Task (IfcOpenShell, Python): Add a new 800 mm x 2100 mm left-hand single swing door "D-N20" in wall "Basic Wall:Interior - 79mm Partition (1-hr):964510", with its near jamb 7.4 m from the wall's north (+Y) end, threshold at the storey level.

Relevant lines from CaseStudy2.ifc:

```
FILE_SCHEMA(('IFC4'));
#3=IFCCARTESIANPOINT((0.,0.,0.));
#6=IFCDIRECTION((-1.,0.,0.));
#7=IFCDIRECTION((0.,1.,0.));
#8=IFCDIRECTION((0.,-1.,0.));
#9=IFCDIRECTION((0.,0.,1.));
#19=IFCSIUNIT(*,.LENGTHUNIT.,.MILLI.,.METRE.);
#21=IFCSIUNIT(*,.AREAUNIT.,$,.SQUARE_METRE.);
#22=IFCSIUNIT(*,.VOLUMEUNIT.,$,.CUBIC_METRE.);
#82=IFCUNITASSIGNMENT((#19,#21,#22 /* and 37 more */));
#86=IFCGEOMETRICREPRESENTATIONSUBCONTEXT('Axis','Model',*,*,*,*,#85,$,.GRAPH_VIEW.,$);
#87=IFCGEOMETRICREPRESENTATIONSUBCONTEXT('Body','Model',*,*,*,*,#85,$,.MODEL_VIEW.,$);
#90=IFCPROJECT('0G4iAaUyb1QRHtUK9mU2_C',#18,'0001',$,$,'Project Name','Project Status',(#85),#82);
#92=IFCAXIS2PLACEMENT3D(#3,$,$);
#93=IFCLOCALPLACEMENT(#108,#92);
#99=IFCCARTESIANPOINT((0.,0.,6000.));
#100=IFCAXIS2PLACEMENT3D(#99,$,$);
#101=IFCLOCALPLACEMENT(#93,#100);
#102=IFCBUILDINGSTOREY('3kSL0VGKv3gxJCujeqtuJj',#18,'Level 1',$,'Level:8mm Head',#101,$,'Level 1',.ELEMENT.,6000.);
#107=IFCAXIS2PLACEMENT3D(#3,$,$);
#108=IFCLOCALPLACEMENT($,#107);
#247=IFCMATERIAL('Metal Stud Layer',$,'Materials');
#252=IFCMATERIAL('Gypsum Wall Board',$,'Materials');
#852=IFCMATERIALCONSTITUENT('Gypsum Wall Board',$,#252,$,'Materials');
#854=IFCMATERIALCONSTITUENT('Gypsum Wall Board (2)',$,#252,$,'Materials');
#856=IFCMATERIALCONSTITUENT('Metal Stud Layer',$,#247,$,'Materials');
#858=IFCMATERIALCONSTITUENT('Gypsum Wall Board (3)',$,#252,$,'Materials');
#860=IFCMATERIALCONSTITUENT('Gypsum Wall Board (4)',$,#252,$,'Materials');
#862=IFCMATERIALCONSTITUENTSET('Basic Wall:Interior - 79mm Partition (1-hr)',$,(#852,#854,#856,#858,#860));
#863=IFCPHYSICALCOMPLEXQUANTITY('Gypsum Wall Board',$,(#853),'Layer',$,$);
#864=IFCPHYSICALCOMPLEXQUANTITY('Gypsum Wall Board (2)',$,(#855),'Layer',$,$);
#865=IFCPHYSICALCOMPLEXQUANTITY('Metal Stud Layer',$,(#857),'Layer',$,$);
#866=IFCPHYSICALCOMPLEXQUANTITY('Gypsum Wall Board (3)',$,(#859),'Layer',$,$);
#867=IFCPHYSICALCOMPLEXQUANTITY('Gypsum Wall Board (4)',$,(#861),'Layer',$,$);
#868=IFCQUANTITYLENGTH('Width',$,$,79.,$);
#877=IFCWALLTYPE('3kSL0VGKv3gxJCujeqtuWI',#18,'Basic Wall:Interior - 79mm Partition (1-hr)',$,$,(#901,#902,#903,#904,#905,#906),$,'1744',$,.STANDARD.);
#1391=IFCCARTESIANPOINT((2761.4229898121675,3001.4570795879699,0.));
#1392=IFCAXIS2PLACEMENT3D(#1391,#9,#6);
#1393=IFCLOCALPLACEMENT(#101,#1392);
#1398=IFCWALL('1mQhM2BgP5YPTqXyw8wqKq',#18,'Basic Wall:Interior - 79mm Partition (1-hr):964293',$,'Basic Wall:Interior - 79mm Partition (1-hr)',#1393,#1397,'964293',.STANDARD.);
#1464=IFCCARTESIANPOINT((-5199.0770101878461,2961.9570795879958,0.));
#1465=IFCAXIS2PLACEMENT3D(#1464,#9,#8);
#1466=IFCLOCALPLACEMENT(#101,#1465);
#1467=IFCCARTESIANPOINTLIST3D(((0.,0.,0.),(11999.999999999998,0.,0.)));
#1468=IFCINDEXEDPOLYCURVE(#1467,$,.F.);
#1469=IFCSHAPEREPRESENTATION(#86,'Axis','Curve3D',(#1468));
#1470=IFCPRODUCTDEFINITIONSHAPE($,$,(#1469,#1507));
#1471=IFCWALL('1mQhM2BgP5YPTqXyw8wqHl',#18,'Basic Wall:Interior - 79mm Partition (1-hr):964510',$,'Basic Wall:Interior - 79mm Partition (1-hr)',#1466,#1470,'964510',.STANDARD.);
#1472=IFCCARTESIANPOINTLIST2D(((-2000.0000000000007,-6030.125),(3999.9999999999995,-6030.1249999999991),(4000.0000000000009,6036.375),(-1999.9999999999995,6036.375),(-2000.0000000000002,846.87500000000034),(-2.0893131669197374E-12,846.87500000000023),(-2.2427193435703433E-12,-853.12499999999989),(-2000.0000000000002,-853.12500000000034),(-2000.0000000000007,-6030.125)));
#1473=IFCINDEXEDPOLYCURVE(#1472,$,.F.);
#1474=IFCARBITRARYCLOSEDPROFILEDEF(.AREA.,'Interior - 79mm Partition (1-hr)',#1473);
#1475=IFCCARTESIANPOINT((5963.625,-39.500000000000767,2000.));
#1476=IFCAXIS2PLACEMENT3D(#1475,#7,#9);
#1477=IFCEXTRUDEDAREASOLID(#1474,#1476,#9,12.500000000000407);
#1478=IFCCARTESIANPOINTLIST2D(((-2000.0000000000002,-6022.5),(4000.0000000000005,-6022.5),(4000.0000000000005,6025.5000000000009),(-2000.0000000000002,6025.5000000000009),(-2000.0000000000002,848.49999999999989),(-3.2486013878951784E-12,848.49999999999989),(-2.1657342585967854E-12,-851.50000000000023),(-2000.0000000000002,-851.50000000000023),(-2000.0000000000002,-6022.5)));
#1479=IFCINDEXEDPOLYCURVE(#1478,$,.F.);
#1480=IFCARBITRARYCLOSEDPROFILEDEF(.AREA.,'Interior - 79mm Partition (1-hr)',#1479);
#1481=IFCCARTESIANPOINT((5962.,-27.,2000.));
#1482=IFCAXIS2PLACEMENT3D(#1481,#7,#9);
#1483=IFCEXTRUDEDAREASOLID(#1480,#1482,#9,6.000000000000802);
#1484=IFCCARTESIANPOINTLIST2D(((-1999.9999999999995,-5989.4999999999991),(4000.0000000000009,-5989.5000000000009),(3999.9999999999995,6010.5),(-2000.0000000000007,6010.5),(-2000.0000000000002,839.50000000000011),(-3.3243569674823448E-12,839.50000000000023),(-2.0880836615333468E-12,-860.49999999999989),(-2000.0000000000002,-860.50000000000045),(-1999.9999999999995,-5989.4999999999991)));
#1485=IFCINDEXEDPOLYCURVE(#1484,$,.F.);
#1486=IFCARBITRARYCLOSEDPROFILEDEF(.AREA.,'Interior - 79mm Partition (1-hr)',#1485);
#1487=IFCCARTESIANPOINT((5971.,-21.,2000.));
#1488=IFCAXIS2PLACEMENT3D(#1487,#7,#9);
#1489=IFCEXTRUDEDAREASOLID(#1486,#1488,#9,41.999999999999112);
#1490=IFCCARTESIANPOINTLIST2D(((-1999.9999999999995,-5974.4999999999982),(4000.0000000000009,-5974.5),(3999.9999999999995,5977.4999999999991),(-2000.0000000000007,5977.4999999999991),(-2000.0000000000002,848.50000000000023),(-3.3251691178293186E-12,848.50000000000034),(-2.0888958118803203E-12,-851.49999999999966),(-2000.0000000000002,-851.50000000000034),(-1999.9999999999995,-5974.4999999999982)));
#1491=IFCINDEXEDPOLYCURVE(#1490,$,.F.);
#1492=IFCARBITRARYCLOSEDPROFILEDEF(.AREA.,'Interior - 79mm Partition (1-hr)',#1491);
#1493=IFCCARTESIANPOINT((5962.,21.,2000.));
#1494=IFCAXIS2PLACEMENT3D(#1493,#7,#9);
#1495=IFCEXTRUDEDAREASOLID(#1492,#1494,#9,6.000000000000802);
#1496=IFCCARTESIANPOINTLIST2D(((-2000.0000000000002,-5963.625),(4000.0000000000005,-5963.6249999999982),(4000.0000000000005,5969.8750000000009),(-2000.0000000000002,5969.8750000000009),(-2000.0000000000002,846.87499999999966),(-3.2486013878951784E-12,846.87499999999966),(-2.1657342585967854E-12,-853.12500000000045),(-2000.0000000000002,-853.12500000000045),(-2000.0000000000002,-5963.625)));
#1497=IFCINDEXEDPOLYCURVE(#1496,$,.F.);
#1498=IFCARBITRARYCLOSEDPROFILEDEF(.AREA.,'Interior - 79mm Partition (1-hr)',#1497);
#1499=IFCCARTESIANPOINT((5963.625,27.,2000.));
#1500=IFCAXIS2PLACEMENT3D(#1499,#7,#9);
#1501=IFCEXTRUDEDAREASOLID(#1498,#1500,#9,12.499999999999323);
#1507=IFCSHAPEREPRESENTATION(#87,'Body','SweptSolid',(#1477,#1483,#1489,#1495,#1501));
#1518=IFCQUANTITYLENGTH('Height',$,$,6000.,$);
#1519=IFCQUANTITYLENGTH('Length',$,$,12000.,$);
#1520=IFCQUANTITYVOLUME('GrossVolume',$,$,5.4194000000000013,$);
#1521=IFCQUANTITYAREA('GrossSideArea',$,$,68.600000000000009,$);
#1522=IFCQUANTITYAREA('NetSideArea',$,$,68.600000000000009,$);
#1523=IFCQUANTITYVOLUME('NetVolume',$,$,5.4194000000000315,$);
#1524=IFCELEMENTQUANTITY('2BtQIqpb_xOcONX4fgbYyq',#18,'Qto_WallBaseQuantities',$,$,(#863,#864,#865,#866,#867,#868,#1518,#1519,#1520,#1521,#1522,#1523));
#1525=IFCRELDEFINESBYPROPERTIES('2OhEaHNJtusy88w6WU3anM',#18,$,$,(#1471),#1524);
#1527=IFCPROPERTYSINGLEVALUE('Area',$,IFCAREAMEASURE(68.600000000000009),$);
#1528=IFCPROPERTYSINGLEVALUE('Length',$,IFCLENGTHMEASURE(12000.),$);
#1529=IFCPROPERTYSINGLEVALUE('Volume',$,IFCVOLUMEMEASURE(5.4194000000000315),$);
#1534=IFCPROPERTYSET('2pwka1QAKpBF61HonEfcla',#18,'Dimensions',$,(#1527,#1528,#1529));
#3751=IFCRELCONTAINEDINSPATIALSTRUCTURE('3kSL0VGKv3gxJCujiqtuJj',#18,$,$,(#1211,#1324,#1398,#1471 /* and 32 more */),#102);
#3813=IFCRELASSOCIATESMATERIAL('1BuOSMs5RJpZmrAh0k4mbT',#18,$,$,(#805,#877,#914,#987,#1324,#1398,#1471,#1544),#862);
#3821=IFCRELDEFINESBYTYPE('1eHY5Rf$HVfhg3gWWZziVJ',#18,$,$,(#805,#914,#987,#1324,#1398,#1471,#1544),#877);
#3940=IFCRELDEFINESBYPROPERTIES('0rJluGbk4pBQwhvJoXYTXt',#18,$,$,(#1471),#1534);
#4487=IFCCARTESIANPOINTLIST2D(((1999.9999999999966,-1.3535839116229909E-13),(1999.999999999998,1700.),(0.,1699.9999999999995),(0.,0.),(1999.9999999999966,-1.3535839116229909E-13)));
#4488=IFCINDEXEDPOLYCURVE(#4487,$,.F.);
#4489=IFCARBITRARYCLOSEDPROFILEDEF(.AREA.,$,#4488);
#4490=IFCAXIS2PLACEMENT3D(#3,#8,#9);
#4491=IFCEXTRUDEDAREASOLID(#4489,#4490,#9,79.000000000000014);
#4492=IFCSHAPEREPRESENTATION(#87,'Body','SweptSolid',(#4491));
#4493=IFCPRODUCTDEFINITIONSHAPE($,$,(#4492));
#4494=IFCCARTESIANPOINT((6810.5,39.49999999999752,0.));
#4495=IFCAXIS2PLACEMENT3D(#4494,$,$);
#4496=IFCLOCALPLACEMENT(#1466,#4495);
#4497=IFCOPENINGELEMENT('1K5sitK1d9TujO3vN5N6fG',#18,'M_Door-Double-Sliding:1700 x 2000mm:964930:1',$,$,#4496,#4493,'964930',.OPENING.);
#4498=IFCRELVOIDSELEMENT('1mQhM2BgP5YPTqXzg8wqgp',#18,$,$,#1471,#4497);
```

```python
import numpy as np
import ifcopenshell
import ifcopenshell.api.feature
import ifcopenshell.api.geometry
import ifcopenshell.api.pset
import ifcopenshell.api.root
import ifcopenshell.api.spatial
import ifcopenshell.geom
import ifcopenshell.util.element
import ifcopenshell.util.placement
import ifcopenshell.util.representation
import ifcopenshell.util.shape
import ifcopenshell.util.unit

model = ifcopenshell.open("CaseStudy2.ifc")
unit_scale = ifcopenshell.util.unit.calculate_unit_scale(model)
area_scale = ifcopenshell.util.unit.calculate_unit_scale(model, "AREAUNIT")
volume_scale = ifcopenshell.util.unit.calculate_unit_scale(model, "VOLUMEUNIT")
settings = ifcopenshell.geom.settings()


def volume(element):
    """Net volume in cubic metres, openings subtracted."""
    shape = ifcopenshell.geom.create_shape(settings, element)
    return ifcopenshell.util.shape.get_volume(shape.geometry)


wall = model.by_id(1471)
storey = ifcopenshell.util.element.get_container(wall, ifc_class="IfcBuildingStorey")
context = ifcopenshell.util.representation.get_context(model, "Model", "Body", "MODEL_VIEW")
before = volume(wall)

width, height, from_end, sill = 0.8, 2.1, 7.4, 0.0  # metres

# The wall runs along its own X axis, and the end named is its -X end.
wall_shape = ifcopenshell.geom.create_shape(settings, wall)
x, y, z = ifcopenshell.util.shape.get_vertices(wall_shape.geometry).T
start = x.min() + from_end
face, thickness = float(y.min()), float(y.max() - y.min())
wall_matrix = ifcopenshell.util.placement.get_local_placement(wall.ObjectPlacement)
level = ifcopenshell.util.placement.get_local_placement(storey.ObjectPlacement)[2, 3]


def in_wall(x, y):
    """Placement at x, y metres in the wall's axes, at sill height."""
    matrix = wall_matrix.copy()
    matrix[:, 3] = wall_matrix @ np.array([x / unit_scale, y / unit_scale, 0.0, 1.0])
    matrix[2, 3] = level + sill / unit_scale
    return matrix


# Opening: a box that overshoots both wall faces by 50 mm.
opening = ifcopenshell.api.root.create_entity(model, ifc_class="IfcOpeningElement", predefined_type="OPENING")
box = ifcopenshell.api.geometry.add_wall_representation(
    model, context=context, length=width, height=height, thickness=thickness + 0.1
)
ifcopenshell.api.geometry.assign_representation(model, product=opening, representation=box)
ifcopenshell.api.geometry.edit_object_placement(model, product=opening, matrix=in_wall(start, face - 0.05), is_si=False)
ifcopenshell.api.feature.add_feature(model, feature=opening, element=wall)

door = ifcopenshell.api.root.create_entity(model, ifc_class="IfcDoor", name="D-N20", predefined_type="DOOR")
door.OverallWidth, door.OverallHeight = width / unit_scale, height / unit_scale
door.OperationType = "SINGLE_SWING_LEFT"
body = ifcopenshell.api.geometry.add_door_representation(
    model,
    context=context,
    overall_width=door.OverallWidth,
    overall_height=door.OverallHeight,
    operation_type="SINGLE_SWING_LEFT",
    lining_properties={"LiningDepth": thickness / unit_scale, "ThresholdDepth": thickness / unit_scale},
)
ifcopenshell.api.geometry.assign_representation(model, product=door, representation=body)
ifcopenshell.api.spatial.assign_container(model, products=[door], relating_structure=storey)
ifcopenshell.api.feature.add_filling(model, opening=opening, element=door)

# The lining spans the wall, so the door starts at the wall face.
ifcopenshell.api.geometry.edit_object_placement(model, product=door, matrix=in_wall(start, face), is_si=False)

after = volume(wall)

# Update the wall's stored quantities.
qto = model.by_id(ifcopenshell.util.element.get_pset(wall, "Qto_WallBaseQuantities", should_inherit=False)["id"])
ifcopenshell.api.pset.edit_qto(model, qto=qto, properties={
    "NetSideArea": after / thickness / area_scale,
    "NetVolume": after / volume_scale,
})
pset = model.by_id(ifcopenshell.util.element.get_pset(wall, "Dimensions", should_inherit=False)["id"])
ifcopenshell.api.pset.edit_pset(model, pset=pset, properties={
    "Area": model.create_entity("IfcAreaMeasure", after / thickness / area_scale),
    "Volume": model.create_entity("IfcVolumeMeasure", after / volume_scale),
})

print(f"wall volume {before:.3f} -> {after:.3f} m3")

model.write("CaseStudy2_rev.ifc")
```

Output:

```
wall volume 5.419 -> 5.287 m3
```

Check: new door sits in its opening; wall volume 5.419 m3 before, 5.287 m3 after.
